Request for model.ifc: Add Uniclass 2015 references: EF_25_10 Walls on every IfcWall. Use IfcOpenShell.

First a look at what the model holds.

```python
import ifcopenshell

model = ifcopenshell.open("model.ifc")
print(model.schema)
print("classifications:", [c.Name for c in model.by_type("IfcClassification")])
for ifc_class in ("IfcDoor", "IfcRoof", "IfcStair", "IfcWall", "IfcWindow"):
    print(ifc_class, len(model.by_type(ifc_class)))
```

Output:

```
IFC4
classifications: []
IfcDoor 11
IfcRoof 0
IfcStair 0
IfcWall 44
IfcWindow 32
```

```python
import ifcopenshell
import ifcopenshell.api.classification

model = ifcopenshell.open("model.ifc")

system = ifcopenshell.api.classification.add_classification(model, classification="Uniclass 2015")

codes = {
    "IfcWall": ("EF_25_10", "Walls"),
}
for ifc_class, (code, name) in codes.items():
    products = model.by_type(ifc_class)
    ifcopenshell.api.classification.add_reference(
        model, products=products, classification=system, identification=code, name=name
    )
    print(code, len(products))

model.write("model-out.ifc")
```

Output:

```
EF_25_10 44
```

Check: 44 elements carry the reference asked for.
